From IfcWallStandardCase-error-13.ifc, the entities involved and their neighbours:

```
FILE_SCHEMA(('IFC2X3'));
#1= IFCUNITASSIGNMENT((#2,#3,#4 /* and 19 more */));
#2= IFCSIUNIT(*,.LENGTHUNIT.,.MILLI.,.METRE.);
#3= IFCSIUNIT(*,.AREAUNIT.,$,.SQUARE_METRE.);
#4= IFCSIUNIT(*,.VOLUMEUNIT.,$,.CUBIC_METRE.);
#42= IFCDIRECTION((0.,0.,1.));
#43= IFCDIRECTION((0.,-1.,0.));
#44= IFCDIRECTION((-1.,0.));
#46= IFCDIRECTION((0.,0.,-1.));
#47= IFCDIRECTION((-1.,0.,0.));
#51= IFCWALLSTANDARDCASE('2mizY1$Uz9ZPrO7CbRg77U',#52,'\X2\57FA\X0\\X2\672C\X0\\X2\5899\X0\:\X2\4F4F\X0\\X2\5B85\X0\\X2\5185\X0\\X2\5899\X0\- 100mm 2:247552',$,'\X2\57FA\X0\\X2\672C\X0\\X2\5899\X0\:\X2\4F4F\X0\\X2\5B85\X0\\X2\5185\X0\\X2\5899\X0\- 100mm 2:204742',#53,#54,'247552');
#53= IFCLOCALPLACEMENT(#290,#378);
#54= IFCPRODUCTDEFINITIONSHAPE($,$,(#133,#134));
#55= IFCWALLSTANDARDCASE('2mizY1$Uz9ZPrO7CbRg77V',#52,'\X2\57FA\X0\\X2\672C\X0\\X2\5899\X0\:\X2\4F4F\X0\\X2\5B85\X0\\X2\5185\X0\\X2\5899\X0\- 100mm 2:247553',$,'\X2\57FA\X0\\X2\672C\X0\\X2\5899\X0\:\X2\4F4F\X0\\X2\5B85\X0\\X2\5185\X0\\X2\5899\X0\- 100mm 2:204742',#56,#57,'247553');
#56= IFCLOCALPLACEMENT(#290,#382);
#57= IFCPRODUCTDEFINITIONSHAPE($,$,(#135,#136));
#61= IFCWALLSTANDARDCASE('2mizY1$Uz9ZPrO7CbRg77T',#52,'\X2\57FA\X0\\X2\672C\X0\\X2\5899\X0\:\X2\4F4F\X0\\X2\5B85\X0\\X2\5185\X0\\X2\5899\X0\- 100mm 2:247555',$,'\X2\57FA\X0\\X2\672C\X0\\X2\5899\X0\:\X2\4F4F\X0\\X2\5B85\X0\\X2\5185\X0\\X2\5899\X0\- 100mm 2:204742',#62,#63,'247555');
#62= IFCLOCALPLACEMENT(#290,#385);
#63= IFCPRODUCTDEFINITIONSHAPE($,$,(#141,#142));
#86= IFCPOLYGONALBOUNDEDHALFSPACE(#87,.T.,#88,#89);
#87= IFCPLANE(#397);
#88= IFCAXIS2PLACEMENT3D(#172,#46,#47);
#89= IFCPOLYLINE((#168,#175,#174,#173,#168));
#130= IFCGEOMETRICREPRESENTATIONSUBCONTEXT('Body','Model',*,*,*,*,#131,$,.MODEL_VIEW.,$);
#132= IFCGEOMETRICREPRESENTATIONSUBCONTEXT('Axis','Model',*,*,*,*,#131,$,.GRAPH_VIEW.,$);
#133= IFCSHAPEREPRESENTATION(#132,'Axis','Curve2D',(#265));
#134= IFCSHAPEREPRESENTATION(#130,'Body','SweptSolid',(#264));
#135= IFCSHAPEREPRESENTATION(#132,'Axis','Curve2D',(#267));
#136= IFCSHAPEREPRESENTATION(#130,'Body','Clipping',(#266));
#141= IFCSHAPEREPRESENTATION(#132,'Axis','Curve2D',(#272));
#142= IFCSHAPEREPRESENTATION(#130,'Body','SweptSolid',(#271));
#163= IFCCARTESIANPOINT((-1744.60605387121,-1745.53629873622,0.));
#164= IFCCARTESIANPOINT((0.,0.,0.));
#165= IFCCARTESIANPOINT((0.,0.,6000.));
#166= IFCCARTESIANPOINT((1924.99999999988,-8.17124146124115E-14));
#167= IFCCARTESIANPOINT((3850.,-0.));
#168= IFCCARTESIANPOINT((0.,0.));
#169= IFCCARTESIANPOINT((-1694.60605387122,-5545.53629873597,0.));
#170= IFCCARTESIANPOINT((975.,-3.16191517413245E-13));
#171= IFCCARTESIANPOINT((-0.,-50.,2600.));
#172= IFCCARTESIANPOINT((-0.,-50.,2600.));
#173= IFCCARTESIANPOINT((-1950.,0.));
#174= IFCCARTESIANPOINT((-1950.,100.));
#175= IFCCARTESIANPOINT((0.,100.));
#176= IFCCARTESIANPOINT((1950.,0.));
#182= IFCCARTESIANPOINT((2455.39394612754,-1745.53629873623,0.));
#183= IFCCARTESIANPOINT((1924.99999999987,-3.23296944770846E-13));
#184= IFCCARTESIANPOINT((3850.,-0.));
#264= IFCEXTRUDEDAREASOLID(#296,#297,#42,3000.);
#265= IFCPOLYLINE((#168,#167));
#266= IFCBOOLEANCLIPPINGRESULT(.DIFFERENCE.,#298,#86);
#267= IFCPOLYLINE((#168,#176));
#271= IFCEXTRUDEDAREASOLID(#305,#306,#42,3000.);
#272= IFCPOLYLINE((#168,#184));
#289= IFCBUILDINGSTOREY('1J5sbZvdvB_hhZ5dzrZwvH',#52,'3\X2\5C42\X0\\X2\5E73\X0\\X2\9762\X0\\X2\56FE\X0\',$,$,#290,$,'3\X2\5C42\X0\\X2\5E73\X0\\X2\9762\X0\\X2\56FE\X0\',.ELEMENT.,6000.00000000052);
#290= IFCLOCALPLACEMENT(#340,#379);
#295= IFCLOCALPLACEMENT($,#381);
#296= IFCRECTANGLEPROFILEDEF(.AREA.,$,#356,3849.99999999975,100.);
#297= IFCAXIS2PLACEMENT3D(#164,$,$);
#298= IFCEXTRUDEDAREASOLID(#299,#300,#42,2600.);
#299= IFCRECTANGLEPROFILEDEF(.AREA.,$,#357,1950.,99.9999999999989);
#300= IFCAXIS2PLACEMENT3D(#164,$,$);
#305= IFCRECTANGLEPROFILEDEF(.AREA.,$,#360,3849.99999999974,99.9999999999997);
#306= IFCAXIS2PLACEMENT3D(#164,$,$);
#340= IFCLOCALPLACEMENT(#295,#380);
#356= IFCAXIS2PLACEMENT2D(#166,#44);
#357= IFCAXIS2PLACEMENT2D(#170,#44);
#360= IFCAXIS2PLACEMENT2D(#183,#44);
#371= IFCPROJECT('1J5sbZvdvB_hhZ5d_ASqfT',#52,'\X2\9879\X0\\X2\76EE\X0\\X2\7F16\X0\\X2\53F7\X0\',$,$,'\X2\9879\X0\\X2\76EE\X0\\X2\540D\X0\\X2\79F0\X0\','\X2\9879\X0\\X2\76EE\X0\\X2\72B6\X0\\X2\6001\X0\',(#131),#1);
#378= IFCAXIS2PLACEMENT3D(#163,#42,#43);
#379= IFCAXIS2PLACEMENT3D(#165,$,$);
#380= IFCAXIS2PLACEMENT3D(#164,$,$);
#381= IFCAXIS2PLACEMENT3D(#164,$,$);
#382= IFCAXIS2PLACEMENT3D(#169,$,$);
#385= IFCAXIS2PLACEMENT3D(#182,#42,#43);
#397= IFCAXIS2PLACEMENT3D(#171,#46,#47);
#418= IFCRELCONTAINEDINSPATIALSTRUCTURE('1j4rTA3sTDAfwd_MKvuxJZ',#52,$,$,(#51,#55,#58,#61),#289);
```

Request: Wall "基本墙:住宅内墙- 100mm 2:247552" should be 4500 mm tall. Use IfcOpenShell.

```python
import ifcopenshell
import ifcopenshell.geom
import ifcopenshell.util.representation
import ifcopenshell.util.shape

model = ifcopenshell.open("IfcWallStandardCase-error-13.ifc")
settings = ifcopenshell.geom.settings()


def volume(element):
    """Net volume in cubic metres, openings subtracted."""
    shape = ifcopenshell.geom.create_shape(settings, element)
    return ifcopenshell.util.shape.get_volume(shape.geometry)


wall = model.by_id(51)
before = volume(wall)

body = ifcopenshell.util.representation.get_representation(wall, "Model", "Body")
solid = body.Items[0]
old_height = solid.Depth
solid.Depth = 4500.0
after = volume(wall)

print(f"height {old_height:g} -> {solid.Depth:g}, volume {before:.3f} -> {after:.3f} m3")

model.write("IfcWallStandardCase-error-13_v2.ifc")
```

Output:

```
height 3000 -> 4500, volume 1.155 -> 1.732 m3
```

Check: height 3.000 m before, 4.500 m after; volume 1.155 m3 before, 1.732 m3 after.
